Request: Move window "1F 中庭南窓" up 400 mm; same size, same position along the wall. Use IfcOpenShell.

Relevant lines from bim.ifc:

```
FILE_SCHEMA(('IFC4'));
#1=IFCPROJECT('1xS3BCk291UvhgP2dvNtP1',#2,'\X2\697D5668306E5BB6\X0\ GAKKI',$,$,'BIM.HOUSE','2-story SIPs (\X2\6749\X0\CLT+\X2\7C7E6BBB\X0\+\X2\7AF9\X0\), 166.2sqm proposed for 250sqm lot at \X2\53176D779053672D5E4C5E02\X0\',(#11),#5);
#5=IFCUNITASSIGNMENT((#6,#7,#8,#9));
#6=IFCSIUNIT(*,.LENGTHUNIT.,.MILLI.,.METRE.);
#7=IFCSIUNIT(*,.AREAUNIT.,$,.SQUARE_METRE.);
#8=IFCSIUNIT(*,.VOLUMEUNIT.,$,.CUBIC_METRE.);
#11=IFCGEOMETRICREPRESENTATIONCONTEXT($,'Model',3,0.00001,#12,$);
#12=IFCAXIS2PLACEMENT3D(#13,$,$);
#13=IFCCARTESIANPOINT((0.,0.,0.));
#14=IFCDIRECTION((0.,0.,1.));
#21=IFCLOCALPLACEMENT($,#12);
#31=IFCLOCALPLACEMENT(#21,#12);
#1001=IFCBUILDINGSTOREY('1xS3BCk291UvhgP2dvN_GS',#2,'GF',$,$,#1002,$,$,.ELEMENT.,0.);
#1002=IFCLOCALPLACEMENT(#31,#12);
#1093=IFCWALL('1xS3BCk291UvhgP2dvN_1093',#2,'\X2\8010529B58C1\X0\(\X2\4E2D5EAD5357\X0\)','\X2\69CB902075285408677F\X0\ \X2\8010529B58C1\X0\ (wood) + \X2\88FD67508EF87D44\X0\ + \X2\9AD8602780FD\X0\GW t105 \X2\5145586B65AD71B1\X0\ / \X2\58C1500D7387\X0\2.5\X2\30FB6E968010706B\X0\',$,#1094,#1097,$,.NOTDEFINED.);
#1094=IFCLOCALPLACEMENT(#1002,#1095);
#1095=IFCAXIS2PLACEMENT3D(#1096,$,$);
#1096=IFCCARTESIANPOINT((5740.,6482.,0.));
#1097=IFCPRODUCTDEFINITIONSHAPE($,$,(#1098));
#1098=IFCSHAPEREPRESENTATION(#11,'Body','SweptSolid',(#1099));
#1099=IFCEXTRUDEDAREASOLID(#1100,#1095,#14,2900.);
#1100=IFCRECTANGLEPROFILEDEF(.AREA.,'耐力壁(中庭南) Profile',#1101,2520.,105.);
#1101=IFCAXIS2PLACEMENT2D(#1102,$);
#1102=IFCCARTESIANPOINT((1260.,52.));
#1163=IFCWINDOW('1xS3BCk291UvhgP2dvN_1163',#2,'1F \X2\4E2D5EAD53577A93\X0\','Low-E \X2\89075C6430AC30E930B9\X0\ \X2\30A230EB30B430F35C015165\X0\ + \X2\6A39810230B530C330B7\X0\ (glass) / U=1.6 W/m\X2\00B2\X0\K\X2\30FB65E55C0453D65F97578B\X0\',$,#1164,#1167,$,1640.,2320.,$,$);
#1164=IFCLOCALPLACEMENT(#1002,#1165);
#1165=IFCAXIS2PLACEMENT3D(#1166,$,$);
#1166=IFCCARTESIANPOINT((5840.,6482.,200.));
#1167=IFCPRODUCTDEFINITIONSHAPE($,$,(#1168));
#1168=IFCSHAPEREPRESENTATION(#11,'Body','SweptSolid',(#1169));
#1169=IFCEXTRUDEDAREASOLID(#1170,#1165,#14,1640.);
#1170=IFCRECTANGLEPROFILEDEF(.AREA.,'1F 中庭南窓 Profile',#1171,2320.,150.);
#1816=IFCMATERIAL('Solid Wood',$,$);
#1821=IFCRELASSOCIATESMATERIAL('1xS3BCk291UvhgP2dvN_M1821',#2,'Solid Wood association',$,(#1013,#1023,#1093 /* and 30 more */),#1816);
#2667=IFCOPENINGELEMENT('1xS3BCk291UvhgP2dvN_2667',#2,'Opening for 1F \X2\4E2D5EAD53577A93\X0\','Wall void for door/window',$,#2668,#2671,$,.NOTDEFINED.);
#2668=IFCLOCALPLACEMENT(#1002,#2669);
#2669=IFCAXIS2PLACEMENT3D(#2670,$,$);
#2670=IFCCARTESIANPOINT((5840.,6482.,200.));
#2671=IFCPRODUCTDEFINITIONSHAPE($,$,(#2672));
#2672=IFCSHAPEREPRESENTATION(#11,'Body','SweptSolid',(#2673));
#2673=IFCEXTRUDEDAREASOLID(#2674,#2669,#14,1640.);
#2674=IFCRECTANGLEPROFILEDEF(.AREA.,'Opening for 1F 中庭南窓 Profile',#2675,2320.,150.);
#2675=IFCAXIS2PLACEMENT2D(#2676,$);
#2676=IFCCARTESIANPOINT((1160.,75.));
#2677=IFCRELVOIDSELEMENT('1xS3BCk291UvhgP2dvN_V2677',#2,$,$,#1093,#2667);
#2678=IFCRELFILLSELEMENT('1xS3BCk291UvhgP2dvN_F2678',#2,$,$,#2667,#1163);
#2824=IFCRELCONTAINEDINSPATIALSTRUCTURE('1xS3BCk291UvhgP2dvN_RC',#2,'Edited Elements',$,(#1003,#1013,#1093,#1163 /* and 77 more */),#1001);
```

```python
import numpy as np
import ifcopenshell
import ifcopenshell.api.geometry
import ifcopenshell.util.placement
import ifcopenshell.util.unit

model = ifcopenshell.open("bim.ifc")
unit_scale = ifcopenshell.util.unit.calculate_unit_scale(model)

window = model.by_guid("1xS3BCk291UvhgP2dvN_1163")
opening = window.FillsVoids[0].RelatingOpeningElement
dz = 400.0

shift = np.array([0.0, 0.0, dz])
# The window is not placed relative to its opening, so move both.
for product in (opening, window):
    matrix = ifcopenshell.util.placement.get_local_placement(product.ObjectPlacement)
    matrix[:3, 3] += shift
    ifcopenshell.api.geometry.edit_object_placement(model, product=product, matrix=matrix, is_si=False)

print(f"moved by {dz * unit_scale:+.3f} m")

model.write("bim_v2.ifc")
```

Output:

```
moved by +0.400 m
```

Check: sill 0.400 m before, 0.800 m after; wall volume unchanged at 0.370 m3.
